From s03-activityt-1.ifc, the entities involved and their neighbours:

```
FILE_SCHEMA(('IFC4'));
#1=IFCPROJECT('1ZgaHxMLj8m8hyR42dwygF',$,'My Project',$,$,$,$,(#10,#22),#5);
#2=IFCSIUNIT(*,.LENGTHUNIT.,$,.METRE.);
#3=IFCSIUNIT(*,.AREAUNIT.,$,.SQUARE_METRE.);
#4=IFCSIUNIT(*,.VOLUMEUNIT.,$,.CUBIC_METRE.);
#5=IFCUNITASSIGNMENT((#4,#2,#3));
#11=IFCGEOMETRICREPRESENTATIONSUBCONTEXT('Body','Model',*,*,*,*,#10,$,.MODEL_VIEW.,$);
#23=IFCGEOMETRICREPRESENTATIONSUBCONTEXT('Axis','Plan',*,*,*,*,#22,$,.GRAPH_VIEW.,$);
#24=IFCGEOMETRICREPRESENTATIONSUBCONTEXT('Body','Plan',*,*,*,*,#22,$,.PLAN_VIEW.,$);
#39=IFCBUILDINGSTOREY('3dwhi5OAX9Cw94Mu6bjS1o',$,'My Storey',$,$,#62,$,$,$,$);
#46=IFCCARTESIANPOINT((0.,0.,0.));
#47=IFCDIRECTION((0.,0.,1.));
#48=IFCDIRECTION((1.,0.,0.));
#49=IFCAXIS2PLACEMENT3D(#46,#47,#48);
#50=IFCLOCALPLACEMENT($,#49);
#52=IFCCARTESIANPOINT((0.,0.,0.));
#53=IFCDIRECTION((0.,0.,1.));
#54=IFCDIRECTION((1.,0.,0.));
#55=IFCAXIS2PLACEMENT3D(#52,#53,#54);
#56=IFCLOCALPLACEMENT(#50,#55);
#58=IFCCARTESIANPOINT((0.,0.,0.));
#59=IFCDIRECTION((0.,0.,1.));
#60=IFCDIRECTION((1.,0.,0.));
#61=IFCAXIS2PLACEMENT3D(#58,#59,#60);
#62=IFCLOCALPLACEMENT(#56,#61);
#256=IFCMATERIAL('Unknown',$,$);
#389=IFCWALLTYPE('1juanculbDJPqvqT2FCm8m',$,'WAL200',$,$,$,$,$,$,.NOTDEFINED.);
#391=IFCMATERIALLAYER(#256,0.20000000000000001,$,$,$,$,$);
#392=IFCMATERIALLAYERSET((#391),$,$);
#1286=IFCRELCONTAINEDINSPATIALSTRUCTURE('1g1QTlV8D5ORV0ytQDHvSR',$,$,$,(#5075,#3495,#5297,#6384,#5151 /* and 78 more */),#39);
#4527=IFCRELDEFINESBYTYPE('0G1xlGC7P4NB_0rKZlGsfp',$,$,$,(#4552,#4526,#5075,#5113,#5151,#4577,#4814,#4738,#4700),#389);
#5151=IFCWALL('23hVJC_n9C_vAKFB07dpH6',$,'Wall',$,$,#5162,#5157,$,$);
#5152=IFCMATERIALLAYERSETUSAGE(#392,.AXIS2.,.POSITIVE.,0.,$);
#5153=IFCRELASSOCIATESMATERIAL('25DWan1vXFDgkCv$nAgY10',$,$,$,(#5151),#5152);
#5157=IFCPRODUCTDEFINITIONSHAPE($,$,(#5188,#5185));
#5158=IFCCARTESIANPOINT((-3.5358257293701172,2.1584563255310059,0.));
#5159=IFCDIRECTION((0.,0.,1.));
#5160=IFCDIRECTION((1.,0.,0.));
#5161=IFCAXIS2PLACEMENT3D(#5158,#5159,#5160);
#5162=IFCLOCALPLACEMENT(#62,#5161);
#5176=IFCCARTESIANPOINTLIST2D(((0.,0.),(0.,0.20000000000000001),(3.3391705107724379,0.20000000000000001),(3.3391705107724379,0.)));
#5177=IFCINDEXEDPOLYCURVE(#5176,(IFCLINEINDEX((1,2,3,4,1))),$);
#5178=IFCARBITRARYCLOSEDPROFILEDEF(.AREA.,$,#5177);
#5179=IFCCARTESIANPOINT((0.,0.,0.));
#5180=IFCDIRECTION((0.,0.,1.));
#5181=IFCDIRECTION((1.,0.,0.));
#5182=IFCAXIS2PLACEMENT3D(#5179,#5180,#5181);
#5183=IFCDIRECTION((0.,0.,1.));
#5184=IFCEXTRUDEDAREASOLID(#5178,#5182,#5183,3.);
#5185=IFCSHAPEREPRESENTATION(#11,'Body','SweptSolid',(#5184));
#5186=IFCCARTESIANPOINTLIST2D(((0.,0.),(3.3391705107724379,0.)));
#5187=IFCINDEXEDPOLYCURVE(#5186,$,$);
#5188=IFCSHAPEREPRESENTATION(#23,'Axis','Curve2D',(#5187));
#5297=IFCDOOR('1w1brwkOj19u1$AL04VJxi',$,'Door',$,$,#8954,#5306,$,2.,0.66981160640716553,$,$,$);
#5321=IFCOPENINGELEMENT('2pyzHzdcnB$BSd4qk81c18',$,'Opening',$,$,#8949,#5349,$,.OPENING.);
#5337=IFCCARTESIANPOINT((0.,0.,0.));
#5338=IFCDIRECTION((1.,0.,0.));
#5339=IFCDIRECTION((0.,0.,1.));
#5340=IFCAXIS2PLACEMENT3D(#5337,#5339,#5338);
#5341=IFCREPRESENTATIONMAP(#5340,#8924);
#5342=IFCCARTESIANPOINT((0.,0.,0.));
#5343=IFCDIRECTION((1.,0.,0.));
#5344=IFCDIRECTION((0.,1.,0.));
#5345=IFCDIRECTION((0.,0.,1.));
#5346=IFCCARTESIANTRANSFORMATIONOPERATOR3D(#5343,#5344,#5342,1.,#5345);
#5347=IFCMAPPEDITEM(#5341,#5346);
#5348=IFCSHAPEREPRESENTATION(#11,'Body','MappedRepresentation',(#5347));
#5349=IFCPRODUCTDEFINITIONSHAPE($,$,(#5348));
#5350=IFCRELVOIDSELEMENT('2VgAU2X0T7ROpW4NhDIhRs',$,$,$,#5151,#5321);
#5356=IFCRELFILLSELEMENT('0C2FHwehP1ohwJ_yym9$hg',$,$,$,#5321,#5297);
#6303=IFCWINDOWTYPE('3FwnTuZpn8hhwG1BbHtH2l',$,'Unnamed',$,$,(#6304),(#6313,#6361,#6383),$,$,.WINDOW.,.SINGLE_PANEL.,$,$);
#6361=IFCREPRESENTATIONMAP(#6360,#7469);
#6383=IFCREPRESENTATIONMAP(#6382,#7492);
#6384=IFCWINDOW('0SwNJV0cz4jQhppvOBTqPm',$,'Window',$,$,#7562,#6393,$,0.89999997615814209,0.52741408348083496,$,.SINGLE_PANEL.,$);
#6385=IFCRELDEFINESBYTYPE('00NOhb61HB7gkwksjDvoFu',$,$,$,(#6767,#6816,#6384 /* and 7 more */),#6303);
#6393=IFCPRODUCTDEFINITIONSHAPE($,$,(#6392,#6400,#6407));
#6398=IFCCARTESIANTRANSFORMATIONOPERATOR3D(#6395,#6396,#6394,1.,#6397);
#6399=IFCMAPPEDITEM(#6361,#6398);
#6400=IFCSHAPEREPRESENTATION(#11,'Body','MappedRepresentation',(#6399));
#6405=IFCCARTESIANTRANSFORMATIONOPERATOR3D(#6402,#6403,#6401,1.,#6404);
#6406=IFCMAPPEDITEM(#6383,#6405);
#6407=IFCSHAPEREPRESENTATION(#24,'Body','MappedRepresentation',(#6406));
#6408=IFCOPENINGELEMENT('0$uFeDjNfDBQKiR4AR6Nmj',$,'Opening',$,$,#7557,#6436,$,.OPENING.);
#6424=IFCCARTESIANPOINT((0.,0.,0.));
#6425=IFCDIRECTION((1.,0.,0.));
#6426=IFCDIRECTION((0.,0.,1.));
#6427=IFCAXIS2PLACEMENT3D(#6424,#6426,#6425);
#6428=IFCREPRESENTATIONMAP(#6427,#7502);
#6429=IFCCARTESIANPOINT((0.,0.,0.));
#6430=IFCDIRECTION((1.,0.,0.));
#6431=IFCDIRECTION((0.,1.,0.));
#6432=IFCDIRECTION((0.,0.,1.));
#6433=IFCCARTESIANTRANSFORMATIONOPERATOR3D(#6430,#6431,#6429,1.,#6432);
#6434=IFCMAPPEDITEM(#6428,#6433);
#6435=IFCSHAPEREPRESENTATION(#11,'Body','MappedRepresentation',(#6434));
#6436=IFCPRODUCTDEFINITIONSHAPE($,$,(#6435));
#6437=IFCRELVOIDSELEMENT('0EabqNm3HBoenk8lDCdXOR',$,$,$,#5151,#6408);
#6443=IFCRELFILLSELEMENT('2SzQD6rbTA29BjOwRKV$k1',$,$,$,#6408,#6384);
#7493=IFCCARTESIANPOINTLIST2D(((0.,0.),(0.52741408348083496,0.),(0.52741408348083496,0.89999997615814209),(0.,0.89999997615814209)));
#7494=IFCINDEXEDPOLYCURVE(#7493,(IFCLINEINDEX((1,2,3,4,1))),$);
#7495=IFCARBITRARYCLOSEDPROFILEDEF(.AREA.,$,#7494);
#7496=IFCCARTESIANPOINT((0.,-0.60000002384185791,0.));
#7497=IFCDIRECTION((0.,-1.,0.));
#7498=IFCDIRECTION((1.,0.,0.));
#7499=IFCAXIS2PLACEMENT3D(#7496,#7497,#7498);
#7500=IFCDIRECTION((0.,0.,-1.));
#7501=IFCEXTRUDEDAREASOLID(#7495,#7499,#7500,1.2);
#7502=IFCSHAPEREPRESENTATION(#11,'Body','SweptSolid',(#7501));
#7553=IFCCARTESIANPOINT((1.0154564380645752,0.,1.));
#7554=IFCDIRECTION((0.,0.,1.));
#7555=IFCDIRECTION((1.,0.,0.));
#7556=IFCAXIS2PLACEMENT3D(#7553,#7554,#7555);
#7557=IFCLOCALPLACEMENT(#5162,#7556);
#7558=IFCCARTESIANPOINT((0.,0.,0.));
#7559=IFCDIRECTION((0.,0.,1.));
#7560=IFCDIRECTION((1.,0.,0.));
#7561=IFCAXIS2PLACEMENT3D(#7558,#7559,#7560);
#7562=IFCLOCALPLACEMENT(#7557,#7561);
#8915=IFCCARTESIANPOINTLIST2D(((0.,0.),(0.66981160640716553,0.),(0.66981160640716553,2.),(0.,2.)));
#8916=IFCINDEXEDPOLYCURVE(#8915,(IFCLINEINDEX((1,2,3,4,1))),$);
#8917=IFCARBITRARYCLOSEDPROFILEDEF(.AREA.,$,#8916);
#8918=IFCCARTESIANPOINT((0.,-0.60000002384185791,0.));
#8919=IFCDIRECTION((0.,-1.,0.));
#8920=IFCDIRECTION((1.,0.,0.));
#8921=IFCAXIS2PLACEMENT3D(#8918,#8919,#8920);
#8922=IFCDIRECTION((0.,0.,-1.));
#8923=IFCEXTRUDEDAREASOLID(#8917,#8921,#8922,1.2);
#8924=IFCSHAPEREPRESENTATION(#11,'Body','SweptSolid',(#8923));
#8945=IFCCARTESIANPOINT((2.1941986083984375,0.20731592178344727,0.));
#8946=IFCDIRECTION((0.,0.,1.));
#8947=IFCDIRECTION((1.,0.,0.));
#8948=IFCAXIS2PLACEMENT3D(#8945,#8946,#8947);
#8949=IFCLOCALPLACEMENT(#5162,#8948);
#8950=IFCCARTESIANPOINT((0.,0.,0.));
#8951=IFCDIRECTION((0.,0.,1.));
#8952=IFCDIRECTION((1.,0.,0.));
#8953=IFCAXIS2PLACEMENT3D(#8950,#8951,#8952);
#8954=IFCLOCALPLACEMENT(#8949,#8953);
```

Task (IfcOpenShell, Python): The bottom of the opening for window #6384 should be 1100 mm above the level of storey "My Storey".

```python
import numpy as np
import ifcopenshell
import ifcopenshell.api.geometry
import ifcopenshell.geom
import ifcopenshell.util.element
import ifcopenshell.util.placement
import ifcopenshell.util.shape
import ifcopenshell.util.unit

model = ifcopenshell.open("s03-activityt-1.ifc")
unit_scale = ifcopenshell.util.unit.calculate_unit_scale(model)

window = model.by_guid("0SwNJV0cz4jQhppvOBTqPm")
opening = window.FillsVoids[0].RelatingOpeningElement
storey = ifcopenshell.util.element.get_container(window, ifc_class="IfcBuildingStorey")
level = ifcopenshell.util.placement.get_local_placement(storey.ObjectPlacement)[2, 3]

# The opening's origin need not be at the sill, so measure its lowest point.
shape = ifcopenshell.geom.create_shape(ifcopenshell.geom.settings(), opening)
bottom = ifcopenshell.util.shape.get_shape_bottom_elevation(shape, shape.geometry) / unit_scale
dz = level + 1.1 / unit_scale - bottom

shift = np.array([0.0, 0.0, dz])
# The window is placed relative to its opening, so it follows when the opening moves.
matrix = ifcopenshell.util.placement.get_local_placement(opening.ObjectPlacement)
matrix[:3, 3] += shift
ifcopenshell.api.geometry.edit_object_placement(
    model, product=opening, matrix=matrix, is_si=False, should_transform_children=True
)

print(f"moved by {dz * unit_scale:+.3f} m")

model.write("s03-activityt-1_v2.ifc")
```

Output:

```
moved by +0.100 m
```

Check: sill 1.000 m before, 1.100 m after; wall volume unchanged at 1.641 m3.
